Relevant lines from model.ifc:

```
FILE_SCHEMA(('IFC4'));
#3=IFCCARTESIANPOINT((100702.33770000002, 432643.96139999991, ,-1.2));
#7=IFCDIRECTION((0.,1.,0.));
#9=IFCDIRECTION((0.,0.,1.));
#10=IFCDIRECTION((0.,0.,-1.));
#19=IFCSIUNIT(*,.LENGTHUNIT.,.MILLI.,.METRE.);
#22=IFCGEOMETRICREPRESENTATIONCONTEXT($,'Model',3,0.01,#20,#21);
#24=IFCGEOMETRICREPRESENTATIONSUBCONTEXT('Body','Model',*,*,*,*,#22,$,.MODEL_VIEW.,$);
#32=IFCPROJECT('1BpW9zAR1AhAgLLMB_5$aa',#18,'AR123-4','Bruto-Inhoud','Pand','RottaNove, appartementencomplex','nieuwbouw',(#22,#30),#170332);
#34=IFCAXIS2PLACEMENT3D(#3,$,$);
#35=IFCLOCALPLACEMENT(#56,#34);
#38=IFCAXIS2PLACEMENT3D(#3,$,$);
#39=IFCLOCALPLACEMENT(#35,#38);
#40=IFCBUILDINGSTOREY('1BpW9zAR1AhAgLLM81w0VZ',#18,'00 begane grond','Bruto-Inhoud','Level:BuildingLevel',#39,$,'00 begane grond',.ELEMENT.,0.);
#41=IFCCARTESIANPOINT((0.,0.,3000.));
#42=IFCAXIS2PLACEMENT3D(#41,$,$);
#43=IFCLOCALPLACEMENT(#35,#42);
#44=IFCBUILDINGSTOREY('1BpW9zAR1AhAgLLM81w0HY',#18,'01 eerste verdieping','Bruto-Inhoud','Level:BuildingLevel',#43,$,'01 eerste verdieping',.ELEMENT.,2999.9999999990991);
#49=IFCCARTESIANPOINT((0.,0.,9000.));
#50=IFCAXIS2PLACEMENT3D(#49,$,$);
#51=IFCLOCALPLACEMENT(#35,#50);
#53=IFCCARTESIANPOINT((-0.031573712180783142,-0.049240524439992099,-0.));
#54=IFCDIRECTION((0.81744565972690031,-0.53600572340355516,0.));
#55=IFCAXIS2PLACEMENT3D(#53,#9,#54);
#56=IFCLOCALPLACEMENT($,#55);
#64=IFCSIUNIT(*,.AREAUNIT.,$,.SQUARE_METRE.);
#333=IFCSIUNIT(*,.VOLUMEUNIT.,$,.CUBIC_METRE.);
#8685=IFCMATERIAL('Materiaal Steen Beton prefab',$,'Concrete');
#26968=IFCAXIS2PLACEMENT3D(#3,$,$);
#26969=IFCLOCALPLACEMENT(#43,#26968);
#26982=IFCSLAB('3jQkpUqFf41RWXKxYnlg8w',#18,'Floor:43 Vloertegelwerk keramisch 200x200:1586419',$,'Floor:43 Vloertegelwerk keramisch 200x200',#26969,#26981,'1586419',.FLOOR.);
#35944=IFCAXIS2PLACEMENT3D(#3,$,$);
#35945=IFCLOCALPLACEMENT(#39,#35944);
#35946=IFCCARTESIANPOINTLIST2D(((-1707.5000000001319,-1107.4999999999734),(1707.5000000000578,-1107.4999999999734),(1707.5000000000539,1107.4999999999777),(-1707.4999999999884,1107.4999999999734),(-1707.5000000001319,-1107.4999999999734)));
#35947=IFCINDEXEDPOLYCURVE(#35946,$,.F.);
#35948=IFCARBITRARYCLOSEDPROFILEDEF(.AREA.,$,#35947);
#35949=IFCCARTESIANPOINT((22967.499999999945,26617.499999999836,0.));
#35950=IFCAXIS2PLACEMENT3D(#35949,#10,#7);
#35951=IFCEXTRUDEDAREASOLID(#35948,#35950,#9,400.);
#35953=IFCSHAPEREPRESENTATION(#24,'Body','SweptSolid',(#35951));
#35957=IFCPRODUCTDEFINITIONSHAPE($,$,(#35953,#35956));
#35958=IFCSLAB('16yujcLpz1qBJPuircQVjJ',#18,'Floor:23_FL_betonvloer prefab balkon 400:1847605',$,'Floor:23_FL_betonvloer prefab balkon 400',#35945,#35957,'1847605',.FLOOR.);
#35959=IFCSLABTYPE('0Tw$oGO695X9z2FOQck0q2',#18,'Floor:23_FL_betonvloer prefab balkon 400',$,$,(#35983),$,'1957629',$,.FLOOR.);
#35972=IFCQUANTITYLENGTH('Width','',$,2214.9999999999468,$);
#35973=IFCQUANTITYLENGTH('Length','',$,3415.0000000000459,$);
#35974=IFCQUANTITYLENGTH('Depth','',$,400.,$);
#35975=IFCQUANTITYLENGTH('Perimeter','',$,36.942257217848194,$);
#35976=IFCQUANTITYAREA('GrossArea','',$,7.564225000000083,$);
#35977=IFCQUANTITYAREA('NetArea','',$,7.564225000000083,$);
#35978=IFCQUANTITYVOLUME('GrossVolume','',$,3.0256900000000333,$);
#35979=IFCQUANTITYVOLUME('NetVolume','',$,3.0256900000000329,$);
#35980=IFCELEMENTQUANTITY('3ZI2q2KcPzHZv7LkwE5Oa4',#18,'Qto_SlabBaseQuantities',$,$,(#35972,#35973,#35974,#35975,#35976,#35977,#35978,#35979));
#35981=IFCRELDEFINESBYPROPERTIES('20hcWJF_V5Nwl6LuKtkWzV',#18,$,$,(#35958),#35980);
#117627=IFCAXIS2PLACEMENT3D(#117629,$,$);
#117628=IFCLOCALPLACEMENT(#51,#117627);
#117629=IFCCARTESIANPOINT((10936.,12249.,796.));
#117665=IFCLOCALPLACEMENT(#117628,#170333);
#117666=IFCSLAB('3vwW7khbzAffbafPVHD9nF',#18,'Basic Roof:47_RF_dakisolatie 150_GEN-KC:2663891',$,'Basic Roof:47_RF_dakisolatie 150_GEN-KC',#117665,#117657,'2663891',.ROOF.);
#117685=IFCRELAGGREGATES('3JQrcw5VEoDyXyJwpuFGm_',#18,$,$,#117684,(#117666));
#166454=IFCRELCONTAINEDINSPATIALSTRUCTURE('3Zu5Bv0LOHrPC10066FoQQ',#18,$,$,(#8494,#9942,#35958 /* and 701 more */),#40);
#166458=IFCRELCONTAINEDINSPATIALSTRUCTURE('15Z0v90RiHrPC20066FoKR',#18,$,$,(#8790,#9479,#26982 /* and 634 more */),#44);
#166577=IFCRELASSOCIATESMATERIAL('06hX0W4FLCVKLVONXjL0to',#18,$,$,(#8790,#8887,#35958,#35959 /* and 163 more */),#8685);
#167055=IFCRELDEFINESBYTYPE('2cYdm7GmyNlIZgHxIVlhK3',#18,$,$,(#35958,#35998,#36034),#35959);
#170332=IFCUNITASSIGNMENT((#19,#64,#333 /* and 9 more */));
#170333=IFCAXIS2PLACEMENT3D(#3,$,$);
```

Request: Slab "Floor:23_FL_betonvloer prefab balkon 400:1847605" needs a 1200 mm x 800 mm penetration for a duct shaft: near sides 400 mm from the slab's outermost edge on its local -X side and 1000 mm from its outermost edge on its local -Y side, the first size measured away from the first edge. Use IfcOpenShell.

```python
import numpy as np
import ifcopenshell
import ifcopenshell.api.feature
import ifcopenshell.api.geometry
import ifcopenshell.api.pset
import ifcopenshell.api.root
import ifcopenshell.geom
import ifcopenshell.util.element
import ifcopenshell.util.placement
import ifcopenshell.util.representation
import ifcopenshell.util.shape
import ifcopenshell.util.unit

model = ifcopenshell.open("model.ifc")
unit_scale = ifcopenshell.util.unit.calculate_unit_scale(model)
area_scale = ifcopenshell.util.unit.calculate_unit_scale(model, "AREAUNIT")
volume_scale = ifcopenshell.util.unit.calculate_unit_scale(model, "VOLUMEUNIT")
settings = ifcopenshell.geom.settings()


def volume(element):
    """Net volume in cubic metres, openings subtracted."""
    shape = ifcopenshell.geom.create_shape(settings, element)
    return ifcopenshell.util.shape.get_volume(shape.geometry)


slab = model.by_guid("16yujcLpz1qBJPuircQVjJ")
before = volume(slab)

# Extent in the slab's own axes, in metres. The edges named are its -X and -Y sides.
slab_shape = ifcopenshell.geom.create_shape(settings, slab)
vertices = ifcopenshell.util.shape.get_vertices(slab_shape.geometry)
x_min, y_min, bottom = vertices.min(axis=0)
top = vertices[:, 2].max()

opening = ifcopenshell.api.root.create_entity(model, ifc_class="IfcOpeningElement", name="Duct shaft opening", predefined_type="OPENING")
context = ifcopenshell.util.representation.get_context(model, "Model", "Body", "MODEL_VIEW")
width, depth = 1.2, 0.8
outline = [(0.0, 0.0), (width, 0.0), (width, depth), (0.0, depth), (0.0, 0.0)]
# Overshoot both faces by 50 mm so the cut is clean.
shape = ifcopenshell.api.geometry.add_slab_representation(
    model, context=context, depth=top - bottom + 0.1, polyline=outline
)
ifcopenshell.api.geometry.assign_representation(model, product=opening, representation=shape)

matrix = ifcopenshell.util.placement.get_local_placement(slab.ObjectPlacement)
matrix[:, 3] = matrix @ np.append(np.array([x_min + 0.4, y_min + 1, bottom - 0.05]) / unit_scale, 1.0)
ifcopenshell.api.geometry.edit_object_placement(model, product=opening, matrix=matrix, is_si=False)
ifcopenshell.api.feature.add_feature(model, feature=opening, element=slab)

after = volume(slab)

# Update the slab's stored quantities.
qto = model.by_id(ifcopenshell.util.element.get_pset(slab, "Qto_SlabBaseQuantities", should_inherit=False)["id"])
ifcopenshell.api.pset.edit_qto(model, qto=qto, properties={
    "NetArea": after / (top - bottom) / area_scale,
    "NetVolume": after / volume_scale,
})

print(f"slab volume {before:.3f} -> {after:.3f} m3")

model.write("model_rev.ifc")
```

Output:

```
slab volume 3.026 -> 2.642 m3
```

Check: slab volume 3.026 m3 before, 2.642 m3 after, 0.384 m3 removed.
